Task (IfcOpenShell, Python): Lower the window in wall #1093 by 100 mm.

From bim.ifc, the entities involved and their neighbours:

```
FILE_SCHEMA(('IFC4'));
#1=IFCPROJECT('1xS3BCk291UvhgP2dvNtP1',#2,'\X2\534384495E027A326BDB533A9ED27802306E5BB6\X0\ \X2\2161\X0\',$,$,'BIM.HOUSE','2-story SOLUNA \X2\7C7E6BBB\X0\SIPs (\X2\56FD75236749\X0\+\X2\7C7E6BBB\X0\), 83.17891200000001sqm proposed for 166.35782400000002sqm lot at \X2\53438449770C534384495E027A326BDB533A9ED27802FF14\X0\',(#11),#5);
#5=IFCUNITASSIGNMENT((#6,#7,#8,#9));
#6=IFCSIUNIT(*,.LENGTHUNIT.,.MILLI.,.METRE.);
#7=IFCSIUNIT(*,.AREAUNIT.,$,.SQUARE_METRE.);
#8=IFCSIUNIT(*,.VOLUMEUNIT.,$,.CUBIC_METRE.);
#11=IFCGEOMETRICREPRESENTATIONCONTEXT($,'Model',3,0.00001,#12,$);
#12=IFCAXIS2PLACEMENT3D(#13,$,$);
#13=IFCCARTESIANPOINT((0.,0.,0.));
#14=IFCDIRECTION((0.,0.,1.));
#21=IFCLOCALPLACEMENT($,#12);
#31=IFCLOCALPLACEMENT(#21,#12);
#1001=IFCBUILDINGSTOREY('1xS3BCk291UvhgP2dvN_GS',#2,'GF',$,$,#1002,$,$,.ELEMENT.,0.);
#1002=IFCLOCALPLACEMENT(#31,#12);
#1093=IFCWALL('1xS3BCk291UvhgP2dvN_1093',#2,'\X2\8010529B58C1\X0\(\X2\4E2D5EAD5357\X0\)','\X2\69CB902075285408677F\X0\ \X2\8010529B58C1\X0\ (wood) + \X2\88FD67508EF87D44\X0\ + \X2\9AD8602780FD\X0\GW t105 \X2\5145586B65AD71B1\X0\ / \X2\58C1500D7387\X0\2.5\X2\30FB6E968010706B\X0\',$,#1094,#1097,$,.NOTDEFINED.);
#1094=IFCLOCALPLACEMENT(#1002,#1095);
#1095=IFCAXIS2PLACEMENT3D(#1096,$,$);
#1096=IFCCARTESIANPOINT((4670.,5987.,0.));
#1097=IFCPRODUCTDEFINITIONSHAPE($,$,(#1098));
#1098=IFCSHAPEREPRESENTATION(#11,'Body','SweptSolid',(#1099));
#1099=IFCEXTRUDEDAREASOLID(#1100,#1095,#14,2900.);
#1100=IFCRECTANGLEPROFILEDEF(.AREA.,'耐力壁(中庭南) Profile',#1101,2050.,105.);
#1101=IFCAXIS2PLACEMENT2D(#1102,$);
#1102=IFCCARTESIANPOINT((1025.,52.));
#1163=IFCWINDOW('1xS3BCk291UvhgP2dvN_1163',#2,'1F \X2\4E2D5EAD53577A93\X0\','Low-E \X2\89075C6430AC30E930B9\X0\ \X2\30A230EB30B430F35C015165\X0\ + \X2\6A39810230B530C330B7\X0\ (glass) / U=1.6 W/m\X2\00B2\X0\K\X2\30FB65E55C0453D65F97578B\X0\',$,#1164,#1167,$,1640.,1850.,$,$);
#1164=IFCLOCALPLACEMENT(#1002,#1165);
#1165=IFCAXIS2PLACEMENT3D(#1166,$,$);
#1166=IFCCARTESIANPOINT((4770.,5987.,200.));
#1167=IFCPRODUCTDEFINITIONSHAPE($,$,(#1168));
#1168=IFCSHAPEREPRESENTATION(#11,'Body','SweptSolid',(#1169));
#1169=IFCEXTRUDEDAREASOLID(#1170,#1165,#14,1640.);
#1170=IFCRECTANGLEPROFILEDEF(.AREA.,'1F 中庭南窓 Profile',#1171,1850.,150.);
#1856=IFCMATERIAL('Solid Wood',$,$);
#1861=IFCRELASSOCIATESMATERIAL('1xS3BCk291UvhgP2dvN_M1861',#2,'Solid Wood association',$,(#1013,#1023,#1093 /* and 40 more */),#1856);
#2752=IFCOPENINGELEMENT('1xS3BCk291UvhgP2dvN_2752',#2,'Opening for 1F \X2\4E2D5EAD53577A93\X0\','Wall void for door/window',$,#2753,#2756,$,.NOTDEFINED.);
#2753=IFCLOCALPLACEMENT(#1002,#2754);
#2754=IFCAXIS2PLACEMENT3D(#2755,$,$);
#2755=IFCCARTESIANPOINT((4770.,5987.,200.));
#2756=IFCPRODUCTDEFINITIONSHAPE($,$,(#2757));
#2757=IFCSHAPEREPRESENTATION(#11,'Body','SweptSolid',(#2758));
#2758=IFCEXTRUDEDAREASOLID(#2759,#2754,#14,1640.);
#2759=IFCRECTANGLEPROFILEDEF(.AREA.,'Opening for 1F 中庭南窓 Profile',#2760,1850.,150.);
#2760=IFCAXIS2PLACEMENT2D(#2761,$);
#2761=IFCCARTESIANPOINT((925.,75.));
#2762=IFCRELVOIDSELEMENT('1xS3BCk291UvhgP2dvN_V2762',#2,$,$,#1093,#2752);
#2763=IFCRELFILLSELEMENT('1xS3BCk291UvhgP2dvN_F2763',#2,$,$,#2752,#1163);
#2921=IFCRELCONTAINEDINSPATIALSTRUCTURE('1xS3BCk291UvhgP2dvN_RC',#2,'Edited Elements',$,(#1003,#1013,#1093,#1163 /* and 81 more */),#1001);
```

```python
import numpy as np
import ifcopenshell
import ifcopenshell.api.geometry
import ifcopenshell.util.placement
import ifcopenshell.util.unit

model = ifcopenshell.open("bim.ifc")
unit_scale = ifcopenshell.util.unit.calculate_unit_scale(model)

window = model.by_guid("1xS3BCk291UvhgP2dvN_1163")
opening = window.FillsVoids[0].RelatingOpeningElement
dz = -0.1 / unit_scale

shift = np.array([0.0, 0.0, dz])
# The window is not placed relative to its opening, so move both.
for product in (opening, window):
    matrix = ifcopenshell.util.placement.get_local_placement(product.ObjectPlacement)
    matrix[:3, 3] += shift
    ifcopenshell.api.geometry.edit_object_placement(model, product=product, matrix=matrix, is_si=False)

print(f"moved by {dz * unit_scale:+.3f} m")

model.write("bim_v2.ifc")
```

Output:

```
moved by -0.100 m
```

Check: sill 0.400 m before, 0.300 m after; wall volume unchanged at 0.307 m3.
